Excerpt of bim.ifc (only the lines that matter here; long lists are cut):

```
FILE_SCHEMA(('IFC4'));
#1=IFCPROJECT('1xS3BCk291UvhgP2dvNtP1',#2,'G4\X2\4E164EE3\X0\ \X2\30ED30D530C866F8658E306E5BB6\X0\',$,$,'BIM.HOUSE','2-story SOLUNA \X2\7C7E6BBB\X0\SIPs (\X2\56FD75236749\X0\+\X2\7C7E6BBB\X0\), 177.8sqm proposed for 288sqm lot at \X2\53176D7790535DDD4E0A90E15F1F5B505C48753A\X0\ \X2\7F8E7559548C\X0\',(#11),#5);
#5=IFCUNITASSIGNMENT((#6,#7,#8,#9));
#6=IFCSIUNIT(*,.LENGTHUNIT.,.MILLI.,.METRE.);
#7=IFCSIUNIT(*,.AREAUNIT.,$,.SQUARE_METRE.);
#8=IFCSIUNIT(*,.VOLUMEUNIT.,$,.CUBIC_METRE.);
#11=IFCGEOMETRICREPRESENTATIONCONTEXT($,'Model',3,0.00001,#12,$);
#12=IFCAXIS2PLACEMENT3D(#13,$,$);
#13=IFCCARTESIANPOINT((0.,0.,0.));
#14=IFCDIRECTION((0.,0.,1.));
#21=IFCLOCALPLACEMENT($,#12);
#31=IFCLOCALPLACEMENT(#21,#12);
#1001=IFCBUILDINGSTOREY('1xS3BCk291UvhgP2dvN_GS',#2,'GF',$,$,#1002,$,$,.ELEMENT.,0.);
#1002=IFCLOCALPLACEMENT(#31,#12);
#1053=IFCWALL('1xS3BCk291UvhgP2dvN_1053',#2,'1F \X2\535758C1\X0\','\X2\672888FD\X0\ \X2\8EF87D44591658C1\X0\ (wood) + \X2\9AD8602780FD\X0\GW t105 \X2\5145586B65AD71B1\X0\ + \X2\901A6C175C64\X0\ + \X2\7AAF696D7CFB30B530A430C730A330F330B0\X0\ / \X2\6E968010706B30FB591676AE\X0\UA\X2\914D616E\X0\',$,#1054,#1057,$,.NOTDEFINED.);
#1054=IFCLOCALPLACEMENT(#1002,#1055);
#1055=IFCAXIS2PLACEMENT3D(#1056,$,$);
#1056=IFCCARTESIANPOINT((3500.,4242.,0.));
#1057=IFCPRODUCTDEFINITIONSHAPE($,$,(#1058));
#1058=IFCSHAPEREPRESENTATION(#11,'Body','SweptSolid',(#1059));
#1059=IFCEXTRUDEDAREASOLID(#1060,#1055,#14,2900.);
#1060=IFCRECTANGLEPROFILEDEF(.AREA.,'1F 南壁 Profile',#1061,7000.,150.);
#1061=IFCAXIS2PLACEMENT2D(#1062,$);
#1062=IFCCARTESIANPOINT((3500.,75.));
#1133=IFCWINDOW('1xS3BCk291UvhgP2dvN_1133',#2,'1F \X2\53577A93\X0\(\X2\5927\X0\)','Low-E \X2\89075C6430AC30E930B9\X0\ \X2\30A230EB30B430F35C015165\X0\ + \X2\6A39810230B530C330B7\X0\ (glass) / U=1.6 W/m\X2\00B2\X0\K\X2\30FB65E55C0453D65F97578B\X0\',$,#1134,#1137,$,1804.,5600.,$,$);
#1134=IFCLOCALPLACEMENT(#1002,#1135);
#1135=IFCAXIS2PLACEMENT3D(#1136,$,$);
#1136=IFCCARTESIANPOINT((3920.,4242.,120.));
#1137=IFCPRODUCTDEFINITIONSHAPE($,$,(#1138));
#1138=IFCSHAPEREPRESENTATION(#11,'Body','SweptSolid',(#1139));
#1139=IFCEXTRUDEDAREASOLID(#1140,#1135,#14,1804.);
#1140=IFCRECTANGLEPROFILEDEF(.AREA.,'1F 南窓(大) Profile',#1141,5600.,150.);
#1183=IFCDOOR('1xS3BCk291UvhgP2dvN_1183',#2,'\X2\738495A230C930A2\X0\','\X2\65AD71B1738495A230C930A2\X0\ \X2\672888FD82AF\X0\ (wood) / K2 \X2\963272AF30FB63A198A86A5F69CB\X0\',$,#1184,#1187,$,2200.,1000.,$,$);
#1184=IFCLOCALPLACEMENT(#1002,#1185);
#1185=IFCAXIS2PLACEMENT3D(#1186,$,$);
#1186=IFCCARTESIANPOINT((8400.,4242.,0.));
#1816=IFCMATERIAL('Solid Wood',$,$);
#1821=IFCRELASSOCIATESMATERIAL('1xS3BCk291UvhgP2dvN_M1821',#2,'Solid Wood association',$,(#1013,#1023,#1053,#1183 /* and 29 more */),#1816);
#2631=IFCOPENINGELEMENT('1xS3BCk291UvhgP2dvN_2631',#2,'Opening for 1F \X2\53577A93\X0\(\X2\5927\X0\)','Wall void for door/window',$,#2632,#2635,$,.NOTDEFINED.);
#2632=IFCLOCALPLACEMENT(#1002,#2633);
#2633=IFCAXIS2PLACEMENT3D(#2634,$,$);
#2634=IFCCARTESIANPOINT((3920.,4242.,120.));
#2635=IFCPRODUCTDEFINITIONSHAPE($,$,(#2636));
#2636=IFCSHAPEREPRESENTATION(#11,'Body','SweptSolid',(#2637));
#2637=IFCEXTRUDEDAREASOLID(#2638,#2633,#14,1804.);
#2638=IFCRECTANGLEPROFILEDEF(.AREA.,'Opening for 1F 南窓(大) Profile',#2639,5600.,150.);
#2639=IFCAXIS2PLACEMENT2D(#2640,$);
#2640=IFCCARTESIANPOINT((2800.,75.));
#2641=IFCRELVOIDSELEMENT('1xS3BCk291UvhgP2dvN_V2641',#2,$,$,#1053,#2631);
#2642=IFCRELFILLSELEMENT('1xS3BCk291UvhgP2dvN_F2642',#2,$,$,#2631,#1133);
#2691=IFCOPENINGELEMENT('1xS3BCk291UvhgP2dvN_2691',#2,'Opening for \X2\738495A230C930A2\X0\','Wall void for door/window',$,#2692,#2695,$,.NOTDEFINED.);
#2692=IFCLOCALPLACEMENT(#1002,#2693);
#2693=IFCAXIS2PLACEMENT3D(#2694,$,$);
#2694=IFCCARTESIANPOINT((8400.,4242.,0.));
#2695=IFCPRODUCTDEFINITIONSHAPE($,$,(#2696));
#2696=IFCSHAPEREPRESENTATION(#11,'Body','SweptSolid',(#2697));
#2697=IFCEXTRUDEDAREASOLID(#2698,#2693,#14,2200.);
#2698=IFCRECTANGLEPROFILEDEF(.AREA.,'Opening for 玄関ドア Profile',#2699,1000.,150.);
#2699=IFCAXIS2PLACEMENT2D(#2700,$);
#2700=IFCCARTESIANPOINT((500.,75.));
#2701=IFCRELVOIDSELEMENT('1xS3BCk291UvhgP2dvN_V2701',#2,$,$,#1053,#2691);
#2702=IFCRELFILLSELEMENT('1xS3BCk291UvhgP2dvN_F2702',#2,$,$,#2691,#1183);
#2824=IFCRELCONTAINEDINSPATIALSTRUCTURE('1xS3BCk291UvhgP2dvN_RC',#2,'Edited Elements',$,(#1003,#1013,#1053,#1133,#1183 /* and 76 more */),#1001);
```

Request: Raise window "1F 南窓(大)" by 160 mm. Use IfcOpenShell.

```python
import numpy as np
import ifcopenshell
import ifcopenshell.api.geometry
import ifcopenshell.util.placement
import ifcopenshell.util.unit

model = ifcopenshell.open("bim.ifc")
unit_scale = ifcopenshell.util.unit.calculate_unit_scale(model)

window = model.by_guid("1xS3BCk291UvhgP2dvN_1133")
opening = window.FillsVoids[0].RelatingOpeningElement
dz = 160.0

shift = np.array([0.0, 0.0, dz])
# The window is not placed relative to its opening, so move both.
for product in (opening, window):
    matrix = ifcopenshell.util.placement.get_local_placement(product.ObjectPlacement)
    matrix[:3, 3] += shift
    ifcopenshell.api.geometry.edit_object_placement(model, product=product, matrix=matrix, is_si=False)

print(f"moved by {dz * unit_scale:+.3f} m")

model.write("bim_edited.ifc")
```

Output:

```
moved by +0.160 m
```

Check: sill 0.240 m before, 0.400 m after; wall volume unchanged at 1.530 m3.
